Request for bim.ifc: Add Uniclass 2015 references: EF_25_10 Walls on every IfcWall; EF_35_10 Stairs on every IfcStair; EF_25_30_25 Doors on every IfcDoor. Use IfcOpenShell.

First a look at what the model holds.

```python
import ifcopenshell

model = ifcopenshell.open("bim.ifc")
print(model.schema)
print("classifications:", [c.Name for c in model.by_type("IfcClassification")])
for ifc_class in ("IfcDoor", "IfcRoof", "IfcStair", "IfcWall", "IfcWindow"):
    print(ifc_class, len(model.by_type(ifc_class)))
```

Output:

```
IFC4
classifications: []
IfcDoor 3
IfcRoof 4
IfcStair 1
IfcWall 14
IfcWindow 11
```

```python
import ifcopenshell
import ifcopenshell.api.classification

model = ifcopenshell.open("bim.ifc")

system = ifcopenshell.api.classification.add_classification(model, classification="Uniclass 2015")

codes = {
    "IfcWall": ("EF_25_10", "Walls"),
    "IfcStair": ("EF_35_10", "Stairs"),
    "IfcDoor": ("EF_25_30_25", "Doors"),
}
for ifc_class, (code, name) in codes.items():
    products = model.by_type(ifc_class)
    ifcopenshell.api.classification.add_reference(
        model, products=products, classification=system, identification=code, name=name
    )
    print(code, len(products))

model.write("bim_edited.ifc")
```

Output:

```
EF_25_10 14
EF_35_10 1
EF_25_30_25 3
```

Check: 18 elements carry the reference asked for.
